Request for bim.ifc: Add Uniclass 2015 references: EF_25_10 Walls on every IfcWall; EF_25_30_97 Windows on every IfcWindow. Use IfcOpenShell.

First a look at what the model holds.

```python
import ifcopenshell

model = ifcopenshell.open("bim.ifc")
print(model.schema)
print("classifications:", [c.Name for c in model.by_type("IfcClassification")])
for ifc_class in ("IfcDoor", "IfcRoof", "IfcStair", "IfcWall", "IfcWindow"):
    print(ifc_class, len(model.by_type(ifc_class)))
```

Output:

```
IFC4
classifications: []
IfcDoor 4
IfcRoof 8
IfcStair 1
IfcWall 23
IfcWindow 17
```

```python
import ifcopenshell
import ifcopenshell.api.classification

model = ifcopenshell.open("bim.ifc")

system = ifcopenshell.api.classification.add_classification(model, classification="Uniclass 2015")

codes = {
    "IfcWall": ("EF_25_10", "Walls"),
    "IfcWindow": ("EF_25_30_97", "Windows"),
}
for ifc_class, (code, name) in codes.items():
    products = model.by_type(ifc_class)
    ifcopenshell.api.classification.add_reference(
        model, products=products, classification=system, identification=code, name=name
    )
    print(code, len(products))

model.write("bim_rev.ifc")
```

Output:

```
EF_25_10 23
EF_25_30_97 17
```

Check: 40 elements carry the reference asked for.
